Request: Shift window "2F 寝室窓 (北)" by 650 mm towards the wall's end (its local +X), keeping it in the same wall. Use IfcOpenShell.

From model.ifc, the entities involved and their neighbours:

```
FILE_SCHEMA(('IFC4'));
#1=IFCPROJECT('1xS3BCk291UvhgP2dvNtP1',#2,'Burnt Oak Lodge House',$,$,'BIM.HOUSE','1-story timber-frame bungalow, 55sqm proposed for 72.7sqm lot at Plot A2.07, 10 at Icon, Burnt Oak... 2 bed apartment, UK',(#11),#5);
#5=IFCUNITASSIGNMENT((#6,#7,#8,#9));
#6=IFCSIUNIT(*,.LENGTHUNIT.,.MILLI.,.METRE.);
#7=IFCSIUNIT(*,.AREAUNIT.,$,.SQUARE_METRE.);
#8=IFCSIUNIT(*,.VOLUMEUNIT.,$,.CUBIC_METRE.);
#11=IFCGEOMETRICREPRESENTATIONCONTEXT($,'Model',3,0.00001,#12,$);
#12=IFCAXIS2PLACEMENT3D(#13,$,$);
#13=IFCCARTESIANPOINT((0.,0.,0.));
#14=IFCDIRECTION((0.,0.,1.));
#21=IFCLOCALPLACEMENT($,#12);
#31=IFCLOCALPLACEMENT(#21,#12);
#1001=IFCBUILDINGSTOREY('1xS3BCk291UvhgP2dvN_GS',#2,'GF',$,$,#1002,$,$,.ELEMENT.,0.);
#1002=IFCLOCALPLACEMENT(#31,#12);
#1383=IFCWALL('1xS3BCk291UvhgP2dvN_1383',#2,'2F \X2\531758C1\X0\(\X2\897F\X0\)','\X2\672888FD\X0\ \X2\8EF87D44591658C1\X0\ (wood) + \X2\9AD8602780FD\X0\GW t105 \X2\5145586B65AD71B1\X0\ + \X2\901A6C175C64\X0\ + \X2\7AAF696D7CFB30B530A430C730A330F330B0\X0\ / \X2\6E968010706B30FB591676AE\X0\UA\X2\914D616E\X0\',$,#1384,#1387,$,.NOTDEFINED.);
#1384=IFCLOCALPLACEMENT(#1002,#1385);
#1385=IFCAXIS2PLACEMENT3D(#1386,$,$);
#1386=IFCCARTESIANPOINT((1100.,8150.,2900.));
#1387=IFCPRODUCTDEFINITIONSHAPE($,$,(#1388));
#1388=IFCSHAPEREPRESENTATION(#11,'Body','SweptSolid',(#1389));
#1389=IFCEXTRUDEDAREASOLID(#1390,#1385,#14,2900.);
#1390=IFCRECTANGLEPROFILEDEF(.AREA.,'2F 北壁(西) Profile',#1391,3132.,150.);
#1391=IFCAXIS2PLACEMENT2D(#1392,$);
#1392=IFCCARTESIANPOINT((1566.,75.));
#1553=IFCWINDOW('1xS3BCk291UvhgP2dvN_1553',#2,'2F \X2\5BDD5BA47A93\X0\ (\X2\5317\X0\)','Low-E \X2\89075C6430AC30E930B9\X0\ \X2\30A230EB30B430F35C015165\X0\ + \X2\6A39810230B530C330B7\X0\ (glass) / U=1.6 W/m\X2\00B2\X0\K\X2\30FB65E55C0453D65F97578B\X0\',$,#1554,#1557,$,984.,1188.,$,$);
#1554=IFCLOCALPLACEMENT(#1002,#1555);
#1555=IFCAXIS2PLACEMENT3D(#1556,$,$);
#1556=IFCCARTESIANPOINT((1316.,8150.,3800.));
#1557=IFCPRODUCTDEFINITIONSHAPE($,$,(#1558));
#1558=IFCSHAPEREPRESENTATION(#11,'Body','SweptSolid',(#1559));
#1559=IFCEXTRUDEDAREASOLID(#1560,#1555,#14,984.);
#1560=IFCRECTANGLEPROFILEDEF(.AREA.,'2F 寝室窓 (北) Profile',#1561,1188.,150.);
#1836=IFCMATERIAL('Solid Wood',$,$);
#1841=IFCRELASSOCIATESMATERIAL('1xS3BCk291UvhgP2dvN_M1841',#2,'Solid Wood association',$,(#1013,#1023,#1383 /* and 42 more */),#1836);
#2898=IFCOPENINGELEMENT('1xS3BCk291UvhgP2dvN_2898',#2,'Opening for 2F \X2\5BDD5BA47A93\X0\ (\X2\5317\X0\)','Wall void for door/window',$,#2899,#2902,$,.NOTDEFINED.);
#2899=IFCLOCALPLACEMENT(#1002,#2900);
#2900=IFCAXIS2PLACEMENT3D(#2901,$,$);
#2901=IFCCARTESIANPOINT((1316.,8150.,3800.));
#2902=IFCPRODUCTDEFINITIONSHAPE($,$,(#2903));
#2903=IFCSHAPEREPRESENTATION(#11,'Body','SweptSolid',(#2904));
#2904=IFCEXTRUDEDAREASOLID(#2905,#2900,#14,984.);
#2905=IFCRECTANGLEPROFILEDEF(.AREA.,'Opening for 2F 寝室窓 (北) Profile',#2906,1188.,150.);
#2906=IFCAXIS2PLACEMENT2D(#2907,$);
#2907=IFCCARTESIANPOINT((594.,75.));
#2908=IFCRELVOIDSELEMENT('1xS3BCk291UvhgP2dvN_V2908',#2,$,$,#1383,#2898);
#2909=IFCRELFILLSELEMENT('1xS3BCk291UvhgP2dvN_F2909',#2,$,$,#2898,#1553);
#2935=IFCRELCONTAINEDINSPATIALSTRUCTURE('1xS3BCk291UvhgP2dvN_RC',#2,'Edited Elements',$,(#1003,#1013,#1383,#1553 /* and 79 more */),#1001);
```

```python
import ifcopenshell
import ifcopenshell.api.geometry
import ifcopenshell.util.placement
import ifcopenshell.util.unit

model = ifcopenshell.open("model.ifc")
unit_scale = ifcopenshell.util.unit.calculate_unit_scale(model)

window = model.by_guid("1xS3BCk291UvhgP2dvN_1553")
opening = window.FillsVoids[0].RelatingOpeningElement
wall = opening.VoidsElements[0].RelatingBuildingElement

wall_matrix = ifcopenshell.util.placement.get_local_placement(wall.ObjectPlacement)
shift = wall_matrix[:3, 0] * 0.65 / unit_scale
before = ifcopenshell.util.placement.get_local_placement(window.ObjectPlacement)[:3, 3].copy()

# The window is not placed relative to its opening, so move both.
for product in (opening, window):
    matrix = ifcopenshell.util.placement.get_local_placement(product.ObjectPlacement)
    matrix[:3, 3] += shift
    ifcopenshell.api.geometry.edit_object_placement(model, product=product, matrix=matrix, is_si=False)

after = ifcopenshell.util.placement.get_local_placement(window.ObjectPlacement)[:3, 3]
print("window moved by", (after - before).round(3) + 0.0)

model.write("model-out.ifc")
```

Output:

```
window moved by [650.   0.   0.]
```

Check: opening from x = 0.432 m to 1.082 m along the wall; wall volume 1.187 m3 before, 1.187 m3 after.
